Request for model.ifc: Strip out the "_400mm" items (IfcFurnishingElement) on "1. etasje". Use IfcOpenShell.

First a look at what the model holds.

```python
import ifcopenshell
import ifcopenshell.util.element

model = ifcopenshell.open("model.ifc")
print(model.schema)
storey = next(s for s in model.by_type("IfcBuildingStorey") if s.Name == "1. etasje")
furniture = [e for e in ifcopenshell.util.element.get_decomposition(storey) if e.is_a("IfcFurnishingElement")]
seen = {}
for e in furniture:
    element_type = ifcopenshell.util.element.get_type(e)
    name = element_type.Name if element_type not in (None, e) else None
    seen[name] = seen.get(name, 0) + 1
for name, count in sorted(seen.items(), key=str):
    print(count, "x", name)
```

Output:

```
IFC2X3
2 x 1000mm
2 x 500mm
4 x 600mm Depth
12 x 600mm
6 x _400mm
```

```python
import ifcopenshell
import ifcopenshell.api.root
import ifcopenshell.util.element

model = ifcopenshell.open("model.ifc")

storey = next(s for s in model.by_type("IfcBuildingStorey") if s.Name == "1. etasje")
furniture = [e for e in ifcopenshell.util.element.get_decomposition(storey) if e.is_a("IfcFurnishingElement")]
targets = [e for e in furniture if (t := ifcopenshell.util.element.get_type(e)) not in (None, e) and t.Name == "_400mm"]

for e in targets:
    ifcopenshell.api.root.remove_product(model, product=e)
print(len(targets), "removed")

model.write("model_rev.ifc")
```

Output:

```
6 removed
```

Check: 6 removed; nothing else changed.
